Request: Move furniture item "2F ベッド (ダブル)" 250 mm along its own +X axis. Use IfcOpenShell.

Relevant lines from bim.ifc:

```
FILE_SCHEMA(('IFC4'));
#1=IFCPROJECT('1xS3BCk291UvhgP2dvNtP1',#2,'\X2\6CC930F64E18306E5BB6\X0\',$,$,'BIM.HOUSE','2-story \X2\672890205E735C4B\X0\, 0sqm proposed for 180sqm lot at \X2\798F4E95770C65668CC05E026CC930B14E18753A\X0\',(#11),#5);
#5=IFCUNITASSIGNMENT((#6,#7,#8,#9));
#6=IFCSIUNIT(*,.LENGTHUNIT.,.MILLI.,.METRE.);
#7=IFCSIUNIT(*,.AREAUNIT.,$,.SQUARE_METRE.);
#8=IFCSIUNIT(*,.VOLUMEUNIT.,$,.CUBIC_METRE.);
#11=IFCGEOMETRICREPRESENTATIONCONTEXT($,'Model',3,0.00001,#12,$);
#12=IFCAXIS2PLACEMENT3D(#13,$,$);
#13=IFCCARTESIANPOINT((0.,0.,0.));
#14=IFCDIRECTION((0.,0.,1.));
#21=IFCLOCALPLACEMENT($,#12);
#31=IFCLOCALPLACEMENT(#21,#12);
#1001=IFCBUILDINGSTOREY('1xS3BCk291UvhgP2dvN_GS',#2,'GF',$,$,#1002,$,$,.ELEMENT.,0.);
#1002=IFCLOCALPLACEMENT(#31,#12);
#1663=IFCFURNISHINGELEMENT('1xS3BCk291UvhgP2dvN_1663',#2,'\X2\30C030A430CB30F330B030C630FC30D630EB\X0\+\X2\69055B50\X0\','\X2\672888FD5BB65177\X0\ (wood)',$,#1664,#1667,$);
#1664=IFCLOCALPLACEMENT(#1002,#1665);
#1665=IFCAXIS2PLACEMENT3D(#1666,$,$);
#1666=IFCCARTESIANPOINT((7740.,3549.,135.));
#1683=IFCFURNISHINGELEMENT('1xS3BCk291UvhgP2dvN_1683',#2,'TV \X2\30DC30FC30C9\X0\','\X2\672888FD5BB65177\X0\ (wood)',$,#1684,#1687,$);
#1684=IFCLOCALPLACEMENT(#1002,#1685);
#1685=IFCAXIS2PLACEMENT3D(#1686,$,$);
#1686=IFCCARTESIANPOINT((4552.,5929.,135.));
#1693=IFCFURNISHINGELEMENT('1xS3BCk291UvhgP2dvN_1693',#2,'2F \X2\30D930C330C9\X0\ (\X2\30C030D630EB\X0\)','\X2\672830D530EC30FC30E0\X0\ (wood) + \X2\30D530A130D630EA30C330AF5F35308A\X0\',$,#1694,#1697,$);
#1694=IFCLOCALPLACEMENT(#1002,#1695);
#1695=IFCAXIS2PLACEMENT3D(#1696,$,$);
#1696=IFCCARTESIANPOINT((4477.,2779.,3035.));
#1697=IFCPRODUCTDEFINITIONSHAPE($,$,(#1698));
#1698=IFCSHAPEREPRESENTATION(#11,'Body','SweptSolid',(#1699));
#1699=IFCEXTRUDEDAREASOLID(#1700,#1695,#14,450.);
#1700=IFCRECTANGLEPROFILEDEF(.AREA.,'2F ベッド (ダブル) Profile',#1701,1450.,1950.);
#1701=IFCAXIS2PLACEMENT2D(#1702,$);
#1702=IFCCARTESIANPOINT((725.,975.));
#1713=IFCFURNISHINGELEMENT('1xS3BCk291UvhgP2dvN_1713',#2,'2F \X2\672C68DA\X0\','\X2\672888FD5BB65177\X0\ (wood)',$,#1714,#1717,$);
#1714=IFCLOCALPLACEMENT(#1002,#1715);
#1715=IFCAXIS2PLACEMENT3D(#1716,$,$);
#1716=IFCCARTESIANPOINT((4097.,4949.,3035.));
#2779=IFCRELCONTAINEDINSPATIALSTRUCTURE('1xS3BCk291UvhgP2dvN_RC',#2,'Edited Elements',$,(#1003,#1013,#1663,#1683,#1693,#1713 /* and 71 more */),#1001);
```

```python
import ifcopenshell
import ifcopenshell.api.geometry
import ifcopenshell.util.placement

model = ifcopenshell.open("bim.ifc")

item = model.by_id(1693)
matrix = ifcopenshell.util.placement.get_local_placement(item.ObjectPlacement)
matrix[:3, 3] += matrix[:3, 0] * 250.0
ifcopenshell.api.geometry.edit_object_placement(model, product=item, matrix=matrix, is_si=False)

print(ifcopenshell.util.placement.get_local_placement(item.ObjectPlacement).round(3) + 0.0)

model.write("bim_updated.ifc")
```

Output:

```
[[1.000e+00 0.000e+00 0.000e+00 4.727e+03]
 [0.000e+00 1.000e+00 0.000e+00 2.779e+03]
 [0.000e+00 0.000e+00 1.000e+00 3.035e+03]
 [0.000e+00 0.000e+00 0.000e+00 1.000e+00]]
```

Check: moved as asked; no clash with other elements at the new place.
